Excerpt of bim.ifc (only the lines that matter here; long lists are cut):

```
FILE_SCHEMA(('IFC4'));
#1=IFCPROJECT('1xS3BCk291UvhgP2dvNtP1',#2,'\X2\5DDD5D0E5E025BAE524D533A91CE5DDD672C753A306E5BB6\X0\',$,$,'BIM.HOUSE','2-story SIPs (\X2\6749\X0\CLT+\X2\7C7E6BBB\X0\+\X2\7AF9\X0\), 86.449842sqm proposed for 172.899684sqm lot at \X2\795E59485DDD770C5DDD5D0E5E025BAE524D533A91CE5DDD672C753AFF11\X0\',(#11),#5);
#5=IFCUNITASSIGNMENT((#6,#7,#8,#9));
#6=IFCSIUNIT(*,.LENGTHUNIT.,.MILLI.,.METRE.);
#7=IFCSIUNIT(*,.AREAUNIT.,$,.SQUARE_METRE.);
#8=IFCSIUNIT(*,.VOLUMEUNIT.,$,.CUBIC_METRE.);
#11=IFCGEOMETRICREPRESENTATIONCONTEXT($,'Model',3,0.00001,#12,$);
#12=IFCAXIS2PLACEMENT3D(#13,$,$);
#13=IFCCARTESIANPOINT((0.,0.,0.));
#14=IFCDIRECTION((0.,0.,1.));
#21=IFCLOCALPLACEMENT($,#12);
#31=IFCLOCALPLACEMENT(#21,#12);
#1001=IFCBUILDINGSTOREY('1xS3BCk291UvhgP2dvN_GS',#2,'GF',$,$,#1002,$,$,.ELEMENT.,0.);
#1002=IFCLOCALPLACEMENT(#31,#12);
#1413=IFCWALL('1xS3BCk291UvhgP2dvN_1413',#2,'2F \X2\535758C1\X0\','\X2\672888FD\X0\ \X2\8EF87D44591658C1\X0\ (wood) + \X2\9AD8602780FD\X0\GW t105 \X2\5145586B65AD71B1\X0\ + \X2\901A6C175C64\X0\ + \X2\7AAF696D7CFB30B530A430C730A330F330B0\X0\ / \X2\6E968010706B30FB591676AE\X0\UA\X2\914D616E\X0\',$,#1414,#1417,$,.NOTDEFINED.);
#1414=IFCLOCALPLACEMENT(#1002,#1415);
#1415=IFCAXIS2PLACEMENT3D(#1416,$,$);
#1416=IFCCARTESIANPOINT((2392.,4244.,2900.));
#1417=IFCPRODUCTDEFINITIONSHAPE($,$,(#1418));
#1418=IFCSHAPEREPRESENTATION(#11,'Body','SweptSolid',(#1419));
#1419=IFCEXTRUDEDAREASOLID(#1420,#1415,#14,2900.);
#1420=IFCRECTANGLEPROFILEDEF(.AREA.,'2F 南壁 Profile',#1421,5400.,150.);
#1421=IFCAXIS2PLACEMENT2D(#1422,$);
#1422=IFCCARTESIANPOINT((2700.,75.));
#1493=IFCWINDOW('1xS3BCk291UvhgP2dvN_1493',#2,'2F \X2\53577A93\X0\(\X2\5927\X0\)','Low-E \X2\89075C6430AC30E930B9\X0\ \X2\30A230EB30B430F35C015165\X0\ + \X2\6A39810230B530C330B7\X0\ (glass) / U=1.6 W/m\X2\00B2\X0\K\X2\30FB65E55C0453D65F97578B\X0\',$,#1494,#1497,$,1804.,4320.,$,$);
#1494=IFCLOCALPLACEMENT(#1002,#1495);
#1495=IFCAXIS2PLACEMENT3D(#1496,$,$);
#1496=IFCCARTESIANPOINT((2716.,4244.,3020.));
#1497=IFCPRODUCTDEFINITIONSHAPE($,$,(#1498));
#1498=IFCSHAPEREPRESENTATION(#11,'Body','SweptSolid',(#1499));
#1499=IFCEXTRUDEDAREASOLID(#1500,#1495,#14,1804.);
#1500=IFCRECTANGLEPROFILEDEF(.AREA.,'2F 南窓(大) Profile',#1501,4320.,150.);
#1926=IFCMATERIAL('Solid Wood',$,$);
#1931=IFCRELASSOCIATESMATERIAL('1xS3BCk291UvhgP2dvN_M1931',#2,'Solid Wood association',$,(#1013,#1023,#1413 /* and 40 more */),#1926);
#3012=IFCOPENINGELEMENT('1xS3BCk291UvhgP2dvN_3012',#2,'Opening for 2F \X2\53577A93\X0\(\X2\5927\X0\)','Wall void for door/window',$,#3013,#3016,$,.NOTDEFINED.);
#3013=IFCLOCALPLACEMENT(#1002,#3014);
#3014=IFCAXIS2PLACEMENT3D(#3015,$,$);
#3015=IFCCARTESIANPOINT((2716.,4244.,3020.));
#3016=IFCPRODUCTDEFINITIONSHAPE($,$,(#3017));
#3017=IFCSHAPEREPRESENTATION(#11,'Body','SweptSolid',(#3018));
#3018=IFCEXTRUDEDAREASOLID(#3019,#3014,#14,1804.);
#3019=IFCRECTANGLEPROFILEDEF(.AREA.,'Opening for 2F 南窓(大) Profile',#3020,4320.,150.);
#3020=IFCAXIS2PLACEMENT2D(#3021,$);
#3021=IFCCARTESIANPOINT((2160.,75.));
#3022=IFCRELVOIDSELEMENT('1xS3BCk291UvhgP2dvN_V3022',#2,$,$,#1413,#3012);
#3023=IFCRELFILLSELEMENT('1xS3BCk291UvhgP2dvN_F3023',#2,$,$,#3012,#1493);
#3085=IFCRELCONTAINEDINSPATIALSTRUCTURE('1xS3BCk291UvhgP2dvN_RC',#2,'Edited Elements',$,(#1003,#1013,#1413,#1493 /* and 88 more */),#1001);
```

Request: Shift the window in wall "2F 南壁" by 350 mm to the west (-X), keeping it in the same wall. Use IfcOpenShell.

```python
import ifcopenshell
import ifcopenshell.api.geometry
import ifcopenshell.util.placement
import ifcopenshell.util.unit

model = ifcopenshell.open("bim.ifc")
unit_scale = ifcopenshell.util.unit.calculate_unit_scale(model)

window = model.by_guid("1xS3BCk291UvhgP2dvN_1493")
opening = window.FillsVoids[0].RelatingOpeningElement
wall = opening.VoidsElements[0].RelatingBuildingElement

wall_matrix = ifcopenshell.util.placement.get_local_placement(wall.ObjectPlacement)
shift = wall_matrix[:3, 0] * -0.35 / unit_scale
before = ifcopenshell.util.placement.get_local_placement(window.ObjectPlacement)[:3, 3].copy()

# The window is not placed relative to its opening, so move both.
for product in (opening, window):
    matrix = ifcopenshell.util.placement.get_local_placement(product.ObjectPlacement)
    matrix[:3, 3] += shift
    ifcopenshell.api.geometry.edit_object_placement(model, product=product, matrix=matrix, is_si=False)

after = ifcopenshell.util.placement.get_local_placement(window.ObjectPlacement)[:3, 3]
print("window moved by", (after - before).round(3) + 0.0)

model.write("bim_v2.ifc")
```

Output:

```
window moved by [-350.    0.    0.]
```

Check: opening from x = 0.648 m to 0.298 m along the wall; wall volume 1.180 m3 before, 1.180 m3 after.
